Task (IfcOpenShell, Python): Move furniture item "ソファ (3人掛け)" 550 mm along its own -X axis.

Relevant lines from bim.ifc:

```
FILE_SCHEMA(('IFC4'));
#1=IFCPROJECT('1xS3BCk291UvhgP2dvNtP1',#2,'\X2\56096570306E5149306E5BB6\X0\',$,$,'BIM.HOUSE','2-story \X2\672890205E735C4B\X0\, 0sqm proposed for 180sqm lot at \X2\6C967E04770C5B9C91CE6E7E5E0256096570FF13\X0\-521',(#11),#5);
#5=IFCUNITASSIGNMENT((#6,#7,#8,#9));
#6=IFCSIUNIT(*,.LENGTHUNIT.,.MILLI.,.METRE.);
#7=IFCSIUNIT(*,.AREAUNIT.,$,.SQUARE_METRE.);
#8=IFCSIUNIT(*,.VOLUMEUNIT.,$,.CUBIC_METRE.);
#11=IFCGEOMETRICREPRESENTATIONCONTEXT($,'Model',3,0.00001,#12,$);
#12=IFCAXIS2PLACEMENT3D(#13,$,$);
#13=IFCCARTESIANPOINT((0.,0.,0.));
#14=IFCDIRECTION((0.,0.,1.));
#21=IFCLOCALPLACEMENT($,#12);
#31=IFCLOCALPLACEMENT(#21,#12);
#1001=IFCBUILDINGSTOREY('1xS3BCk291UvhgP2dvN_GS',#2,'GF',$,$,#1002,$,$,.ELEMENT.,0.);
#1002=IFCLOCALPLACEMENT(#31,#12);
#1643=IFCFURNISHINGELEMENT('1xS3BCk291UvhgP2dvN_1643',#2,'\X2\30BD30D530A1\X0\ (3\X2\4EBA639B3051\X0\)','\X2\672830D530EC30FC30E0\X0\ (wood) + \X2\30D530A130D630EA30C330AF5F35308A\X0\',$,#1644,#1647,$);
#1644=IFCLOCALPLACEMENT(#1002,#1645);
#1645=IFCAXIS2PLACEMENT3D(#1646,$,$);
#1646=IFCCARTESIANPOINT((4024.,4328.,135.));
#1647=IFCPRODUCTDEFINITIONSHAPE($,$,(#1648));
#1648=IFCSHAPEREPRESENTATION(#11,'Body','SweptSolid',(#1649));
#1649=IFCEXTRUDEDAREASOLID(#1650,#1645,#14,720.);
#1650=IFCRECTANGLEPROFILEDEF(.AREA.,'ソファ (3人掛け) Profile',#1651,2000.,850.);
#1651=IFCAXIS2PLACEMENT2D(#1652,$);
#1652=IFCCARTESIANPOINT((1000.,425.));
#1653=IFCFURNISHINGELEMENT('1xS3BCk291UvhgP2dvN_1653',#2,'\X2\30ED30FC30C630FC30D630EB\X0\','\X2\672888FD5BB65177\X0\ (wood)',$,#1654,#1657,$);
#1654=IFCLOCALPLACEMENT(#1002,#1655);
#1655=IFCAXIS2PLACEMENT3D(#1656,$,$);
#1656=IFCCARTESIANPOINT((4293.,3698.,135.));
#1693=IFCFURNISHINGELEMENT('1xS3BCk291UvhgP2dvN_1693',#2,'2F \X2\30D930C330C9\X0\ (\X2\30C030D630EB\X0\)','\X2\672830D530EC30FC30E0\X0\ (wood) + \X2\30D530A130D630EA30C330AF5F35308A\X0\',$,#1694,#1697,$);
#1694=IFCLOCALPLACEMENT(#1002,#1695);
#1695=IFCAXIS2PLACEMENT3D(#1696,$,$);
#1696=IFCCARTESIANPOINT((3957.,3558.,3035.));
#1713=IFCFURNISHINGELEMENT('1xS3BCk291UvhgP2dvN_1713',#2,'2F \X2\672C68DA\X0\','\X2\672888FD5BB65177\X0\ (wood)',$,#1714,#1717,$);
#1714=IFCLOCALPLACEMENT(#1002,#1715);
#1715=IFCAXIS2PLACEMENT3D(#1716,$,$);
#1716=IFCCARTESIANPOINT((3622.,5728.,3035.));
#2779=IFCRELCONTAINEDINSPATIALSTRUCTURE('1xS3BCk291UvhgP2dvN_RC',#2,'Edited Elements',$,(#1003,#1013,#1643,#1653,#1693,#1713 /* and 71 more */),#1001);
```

```python
import ifcopenshell
import ifcopenshell.api.geometry
import ifcopenshell.util.placement

model = ifcopenshell.open("bim.ifc")

item = model.by_guid("1xS3BCk291UvhgP2dvN_1643")
matrix = ifcopenshell.util.placement.get_local_placement(item.ObjectPlacement)
matrix[:3, 3] -= matrix[:3, 0] * 550.0
ifcopenshell.api.geometry.edit_object_placement(model, product=item, matrix=matrix, is_si=False)

print(ifcopenshell.util.placement.get_local_placement(item.ObjectPlacement).round(3) + 0.0)

model.write("bim_updated.ifc")
```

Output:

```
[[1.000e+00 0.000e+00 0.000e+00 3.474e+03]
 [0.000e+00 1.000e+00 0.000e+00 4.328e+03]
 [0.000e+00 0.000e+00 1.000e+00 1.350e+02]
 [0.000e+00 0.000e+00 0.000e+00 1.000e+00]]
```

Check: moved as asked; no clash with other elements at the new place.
